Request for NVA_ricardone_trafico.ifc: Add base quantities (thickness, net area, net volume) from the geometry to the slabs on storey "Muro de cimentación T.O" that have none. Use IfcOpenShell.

First a look at what the model holds.

```python
import ifcopenshell
import ifcopenshell.util.element
import ifcopenshell.util.unit

model = ifcopenshell.open("NVA_ricardone_trafico.ifc")
print(model.schema)
for unit_type in ("LENGTHUNIT", "AREAUNIT", "VOLUMEUNIT"):
    print(unit_type, ifcopenshell.util.unit.calculate_unit_scale(model, unit_type))
storey = next(s for s in model.by_type("IfcBuildingStorey") if s.Name == "Muro de cimentación T.O")
slabs = [e for e in ifcopenshell.util.element.get_decomposition(storey) if e.is_a("IfcSlab")]
for e in sorted(slabs, key=lambda e: e.id()):
    print(e.id(), e.is_a(), e.Name, list(ifcopenshell.util.element.get_psets(e, qtos_only=True)), sep=" | ")
```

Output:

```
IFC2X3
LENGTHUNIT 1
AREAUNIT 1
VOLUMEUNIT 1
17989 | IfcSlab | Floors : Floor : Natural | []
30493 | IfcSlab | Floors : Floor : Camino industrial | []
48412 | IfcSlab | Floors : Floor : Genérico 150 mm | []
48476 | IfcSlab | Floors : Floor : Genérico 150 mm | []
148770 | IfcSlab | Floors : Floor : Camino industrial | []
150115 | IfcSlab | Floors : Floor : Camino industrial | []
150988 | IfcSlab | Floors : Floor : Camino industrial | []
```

```python
import ifcopenshell
import ifcopenshell.api.pset
import ifcopenshell.geom
import ifcopenshell.util.element
import ifcopenshell.util.shape
import ifcopenshell.util.unit

model = ifcopenshell.open("NVA_ricardone_trafico.ifc")
unit_scale = ifcopenshell.util.unit.calculate_unit_scale(model)
area_scale = ifcopenshell.util.unit.calculate_unit_scale(model, "AREAUNIT")
volume_scale = ifcopenshell.util.unit.calculate_unit_scale(model, "VOLUMEUNIT")
settings = ifcopenshell.geom.settings()

storey = next(s for s in model.by_type("IfcBuildingStorey") if s.Name == "Muro de cimentación T.O")
slabs = [e for e in ifcopenshell.util.element.get_decomposition(storey) if e.is_a("IfcSlab")]

for e in sorted(slabs, key=lambda e: e.id()):
    if ifcopenshell.util.element.get_psets(e, qtos_only=True, should_inherit=False):
        continue
    # Geometry comes back in metres, in the element's own axes.
    shape = ifcopenshell.geom.create_shape(settings, e)
    values = {
        "Width": ifcopenshell.util.shape.get_z(shape.geometry) / unit_scale,
        "NetArea": ifcopenshell.util.shape.get_footprint_area(shape.geometry) / area_scale,
        "NetVolume": ifcopenshell.util.shape.get_volume(shape.geometry) / volume_scale,
    }
    qto = ifcopenshell.api.pset.add_qto(model, product=e, name="BaseQuantities")
    ifcopenshell.api.pset.edit_qto(model, qto=qto, properties=values)
    print(e.id(), {k: round(v, 3) for k, v in values.items()})

model.write("NVA_ricardone_trafico_v2.ifc")
```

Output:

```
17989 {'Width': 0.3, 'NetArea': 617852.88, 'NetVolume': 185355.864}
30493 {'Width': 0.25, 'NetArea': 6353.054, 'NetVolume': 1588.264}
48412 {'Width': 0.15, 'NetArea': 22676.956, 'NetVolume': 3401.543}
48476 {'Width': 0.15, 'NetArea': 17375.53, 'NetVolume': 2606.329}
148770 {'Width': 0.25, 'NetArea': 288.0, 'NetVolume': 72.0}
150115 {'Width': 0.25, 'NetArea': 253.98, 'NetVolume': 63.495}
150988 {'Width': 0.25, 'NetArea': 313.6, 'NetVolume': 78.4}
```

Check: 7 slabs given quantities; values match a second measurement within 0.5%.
